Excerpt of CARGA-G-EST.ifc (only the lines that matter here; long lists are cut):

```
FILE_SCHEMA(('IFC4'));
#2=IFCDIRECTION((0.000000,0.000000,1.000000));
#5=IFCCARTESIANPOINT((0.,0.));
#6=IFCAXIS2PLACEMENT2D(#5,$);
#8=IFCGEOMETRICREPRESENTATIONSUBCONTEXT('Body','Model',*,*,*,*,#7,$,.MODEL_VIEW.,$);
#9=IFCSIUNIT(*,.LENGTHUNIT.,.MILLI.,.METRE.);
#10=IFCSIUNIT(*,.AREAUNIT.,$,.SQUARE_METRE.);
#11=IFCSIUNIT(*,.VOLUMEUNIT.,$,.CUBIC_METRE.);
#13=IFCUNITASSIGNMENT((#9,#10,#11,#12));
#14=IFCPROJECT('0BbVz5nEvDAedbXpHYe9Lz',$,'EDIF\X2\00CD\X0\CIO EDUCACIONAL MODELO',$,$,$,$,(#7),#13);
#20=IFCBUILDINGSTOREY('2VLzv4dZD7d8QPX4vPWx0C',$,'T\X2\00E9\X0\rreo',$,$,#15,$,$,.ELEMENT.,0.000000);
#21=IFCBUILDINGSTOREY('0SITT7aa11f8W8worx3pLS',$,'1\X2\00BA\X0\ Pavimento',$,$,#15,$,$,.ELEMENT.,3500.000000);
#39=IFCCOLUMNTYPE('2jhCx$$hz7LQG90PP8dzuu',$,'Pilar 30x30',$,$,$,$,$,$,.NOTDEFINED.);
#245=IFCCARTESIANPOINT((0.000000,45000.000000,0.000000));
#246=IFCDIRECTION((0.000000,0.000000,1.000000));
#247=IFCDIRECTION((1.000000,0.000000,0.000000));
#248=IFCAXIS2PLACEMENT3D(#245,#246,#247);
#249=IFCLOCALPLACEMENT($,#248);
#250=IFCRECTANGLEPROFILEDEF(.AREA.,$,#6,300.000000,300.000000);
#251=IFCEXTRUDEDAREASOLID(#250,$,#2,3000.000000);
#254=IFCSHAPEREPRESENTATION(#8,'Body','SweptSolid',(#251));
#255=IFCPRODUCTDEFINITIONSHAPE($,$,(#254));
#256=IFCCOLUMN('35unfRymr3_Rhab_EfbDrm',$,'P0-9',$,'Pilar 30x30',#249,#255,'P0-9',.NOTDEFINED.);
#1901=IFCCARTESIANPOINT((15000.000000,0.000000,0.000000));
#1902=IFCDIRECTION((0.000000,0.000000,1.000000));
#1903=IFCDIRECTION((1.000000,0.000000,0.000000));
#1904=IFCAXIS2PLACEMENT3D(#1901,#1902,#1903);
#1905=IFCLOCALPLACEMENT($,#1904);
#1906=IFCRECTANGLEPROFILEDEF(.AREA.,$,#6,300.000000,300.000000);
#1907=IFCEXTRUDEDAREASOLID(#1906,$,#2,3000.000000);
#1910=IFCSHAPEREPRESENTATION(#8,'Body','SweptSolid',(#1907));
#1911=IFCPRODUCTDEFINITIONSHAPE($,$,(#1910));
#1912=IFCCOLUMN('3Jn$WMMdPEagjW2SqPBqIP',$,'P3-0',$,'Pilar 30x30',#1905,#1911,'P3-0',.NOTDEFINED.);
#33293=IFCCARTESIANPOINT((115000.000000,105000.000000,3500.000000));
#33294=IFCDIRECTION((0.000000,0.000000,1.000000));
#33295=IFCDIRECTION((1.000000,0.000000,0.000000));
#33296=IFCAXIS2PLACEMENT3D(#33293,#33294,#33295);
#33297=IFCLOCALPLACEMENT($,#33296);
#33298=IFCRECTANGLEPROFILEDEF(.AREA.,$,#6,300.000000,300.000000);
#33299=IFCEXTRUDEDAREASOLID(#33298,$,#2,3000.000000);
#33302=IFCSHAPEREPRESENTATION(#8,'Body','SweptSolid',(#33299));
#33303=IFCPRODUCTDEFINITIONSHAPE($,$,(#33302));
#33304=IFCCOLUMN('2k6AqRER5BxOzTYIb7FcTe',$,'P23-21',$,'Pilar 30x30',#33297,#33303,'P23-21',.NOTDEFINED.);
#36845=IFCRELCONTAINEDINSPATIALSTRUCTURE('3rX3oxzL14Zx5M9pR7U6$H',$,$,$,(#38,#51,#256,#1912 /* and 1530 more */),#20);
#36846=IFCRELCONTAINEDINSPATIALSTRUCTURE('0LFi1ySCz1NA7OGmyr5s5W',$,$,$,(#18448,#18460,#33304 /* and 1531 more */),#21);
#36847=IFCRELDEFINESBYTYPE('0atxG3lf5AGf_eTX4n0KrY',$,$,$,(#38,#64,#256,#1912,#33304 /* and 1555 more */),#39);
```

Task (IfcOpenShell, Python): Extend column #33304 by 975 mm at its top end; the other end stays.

```python
import ifcopenshell
import ifcopenshell.util.representation
import ifcopenshell.util.unit

model = ifcopenshell.open("CARGA-G-EST.ifc")
unit_scale = ifcopenshell.util.unit.calculate_unit_scale(model)

member = model.by_guid("2k6AqRER5BxOzTYIb7FcTe")
change = 0.975 / unit_scale

# The extrusion runs towards the end named, so only its depth changes.
body = ifcopenshell.util.representation.get_representation(member, "Model", "Body")
solid = body.Items[0]
old_length = solid.Depth
solid.Depth += change

print(f"length {old_length:g} -> {solid.Depth:g}")

model.write("CARGA-G-EST_updated.ifc")
```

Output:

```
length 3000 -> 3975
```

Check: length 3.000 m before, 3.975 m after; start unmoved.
